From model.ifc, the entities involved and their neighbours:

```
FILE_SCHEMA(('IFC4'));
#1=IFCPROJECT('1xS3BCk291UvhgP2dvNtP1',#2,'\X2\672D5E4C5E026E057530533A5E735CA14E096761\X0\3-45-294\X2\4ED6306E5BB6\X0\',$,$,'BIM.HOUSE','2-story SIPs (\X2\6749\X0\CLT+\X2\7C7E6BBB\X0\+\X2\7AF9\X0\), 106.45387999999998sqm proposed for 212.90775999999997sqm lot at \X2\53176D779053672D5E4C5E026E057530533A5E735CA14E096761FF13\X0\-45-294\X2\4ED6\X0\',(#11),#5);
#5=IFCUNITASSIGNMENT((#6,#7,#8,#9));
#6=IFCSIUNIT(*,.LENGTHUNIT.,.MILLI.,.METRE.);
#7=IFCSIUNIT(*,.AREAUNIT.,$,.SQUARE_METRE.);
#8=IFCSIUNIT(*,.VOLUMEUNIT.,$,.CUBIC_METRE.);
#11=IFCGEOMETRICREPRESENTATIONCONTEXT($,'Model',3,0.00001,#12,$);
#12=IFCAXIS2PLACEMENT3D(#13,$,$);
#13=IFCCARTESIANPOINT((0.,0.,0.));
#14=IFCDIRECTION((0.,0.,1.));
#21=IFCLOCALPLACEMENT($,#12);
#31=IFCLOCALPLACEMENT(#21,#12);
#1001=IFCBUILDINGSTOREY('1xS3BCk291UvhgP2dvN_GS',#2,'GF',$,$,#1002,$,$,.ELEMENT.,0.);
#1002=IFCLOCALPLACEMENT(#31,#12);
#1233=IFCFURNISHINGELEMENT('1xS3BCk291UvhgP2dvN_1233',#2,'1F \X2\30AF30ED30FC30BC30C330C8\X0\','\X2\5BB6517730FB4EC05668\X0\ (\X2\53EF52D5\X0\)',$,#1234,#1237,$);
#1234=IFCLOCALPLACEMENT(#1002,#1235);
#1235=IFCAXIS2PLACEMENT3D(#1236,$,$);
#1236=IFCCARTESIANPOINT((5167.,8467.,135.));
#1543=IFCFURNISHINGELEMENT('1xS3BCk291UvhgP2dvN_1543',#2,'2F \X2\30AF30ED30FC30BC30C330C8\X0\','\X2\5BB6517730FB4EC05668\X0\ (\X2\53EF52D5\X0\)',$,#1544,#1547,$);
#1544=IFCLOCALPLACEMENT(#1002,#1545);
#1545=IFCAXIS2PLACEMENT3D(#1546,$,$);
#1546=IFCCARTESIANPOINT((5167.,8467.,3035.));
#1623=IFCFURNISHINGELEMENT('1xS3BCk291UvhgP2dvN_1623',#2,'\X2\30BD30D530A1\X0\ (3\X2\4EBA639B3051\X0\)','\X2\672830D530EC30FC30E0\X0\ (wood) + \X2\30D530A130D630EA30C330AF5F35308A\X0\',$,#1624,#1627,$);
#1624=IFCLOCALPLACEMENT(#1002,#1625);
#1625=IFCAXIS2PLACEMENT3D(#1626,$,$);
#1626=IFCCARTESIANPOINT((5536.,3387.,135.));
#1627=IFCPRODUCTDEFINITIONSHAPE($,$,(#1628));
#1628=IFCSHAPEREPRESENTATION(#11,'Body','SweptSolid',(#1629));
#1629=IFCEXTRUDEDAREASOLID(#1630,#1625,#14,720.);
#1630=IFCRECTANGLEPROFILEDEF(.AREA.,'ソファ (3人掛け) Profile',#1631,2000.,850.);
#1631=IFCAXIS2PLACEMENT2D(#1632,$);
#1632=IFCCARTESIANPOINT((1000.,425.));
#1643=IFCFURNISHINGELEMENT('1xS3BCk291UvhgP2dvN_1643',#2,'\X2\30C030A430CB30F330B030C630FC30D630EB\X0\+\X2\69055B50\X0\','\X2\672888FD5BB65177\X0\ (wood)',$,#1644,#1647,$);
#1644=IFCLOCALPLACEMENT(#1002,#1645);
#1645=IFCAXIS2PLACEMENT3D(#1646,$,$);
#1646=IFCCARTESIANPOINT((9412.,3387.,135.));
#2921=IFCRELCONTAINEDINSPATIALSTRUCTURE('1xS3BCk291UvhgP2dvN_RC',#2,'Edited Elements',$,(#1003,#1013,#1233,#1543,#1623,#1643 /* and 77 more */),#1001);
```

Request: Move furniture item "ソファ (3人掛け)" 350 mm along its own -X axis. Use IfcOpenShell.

```python
import ifcopenshell
import ifcopenshell.api.geometry
import ifcopenshell.util.placement
import ifcopenshell.util.unit

model = ifcopenshell.open("model.ifc")
unit_scale = ifcopenshell.util.unit.calculate_unit_scale(model)

item = model.by_guid("1xS3BCk291UvhgP2dvN_1623")
matrix = ifcopenshell.util.placement.get_local_placement(item.ObjectPlacement)
matrix[:3, 3] -= matrix[:3, 0] * 0.35 / unit_scale
ifcopenshell.api.geometry.edit_object_placement(model, product=item, matrix=matrix, is_si=False)

print(ifcopenshell.util.placement.get_local_placement(item.ObjectPlacement).round(3) + 0.0)

model.write("model-out.ifc")
```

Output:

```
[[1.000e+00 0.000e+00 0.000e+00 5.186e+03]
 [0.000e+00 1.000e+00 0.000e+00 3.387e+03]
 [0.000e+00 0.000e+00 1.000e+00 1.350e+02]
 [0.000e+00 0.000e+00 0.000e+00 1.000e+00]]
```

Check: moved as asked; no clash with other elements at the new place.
